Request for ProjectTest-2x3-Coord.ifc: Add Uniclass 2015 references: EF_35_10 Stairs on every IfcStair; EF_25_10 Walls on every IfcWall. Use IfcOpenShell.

First a look at what the model holds.

```python
import ifcopenshell

model = ifcopenshell.open("ProjectTest-2x3-Coord.ifc")
print(model.schema)
print("classifications:", [c.Name for c in model.by_type("IfcClassification")])
for ifc_class in ("IfcDoor", "IfcRoof", "IfcStair", "IfcWall", "IfcWindow"):
    print(ifc_class, len(model.by_type(ifc_class)))
```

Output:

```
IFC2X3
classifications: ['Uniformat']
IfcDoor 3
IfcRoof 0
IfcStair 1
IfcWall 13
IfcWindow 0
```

```python
import ifcopenshell
import ifcopenshell.api.classification

model = ifcopenshell.open("ProjectTest-2x3-Coord.ifc")

# IFC2X3 requires Source and Edition and has no link from the project to the system.
system = model.create_entity("IfcClassification", Source="NBS", Edition="2015", Name="Uniclass 2015")

codes = {
    "IfcStair": ("EF_35_10", "Stairs"),
    "IfcWall": ("EF_25_10", "Walls"),
}
for ifc_class, (code, name) in codes.items():
    products = model.by_type(ifc_class)
    ifcopenshell.api.classification.add_reference(
        model, products=products, classification=system, identification=code, name=name
    )
    print(code, len(products))

model.write("ProjectTest-2x3-Coord_updated.ifc")
```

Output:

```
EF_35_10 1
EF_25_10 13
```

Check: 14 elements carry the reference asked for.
